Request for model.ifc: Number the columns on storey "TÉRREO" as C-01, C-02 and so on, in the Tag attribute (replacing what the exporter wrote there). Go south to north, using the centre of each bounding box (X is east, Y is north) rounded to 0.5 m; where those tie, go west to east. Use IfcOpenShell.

First a look at what the model holds.

```python
import ifcopenshell
import ifcopenshell.util.element
import ifcopenshell.util.placement

model = ifcopenshell.open("model.ifc")
print(model.schema)
storey = next(s for s in model.by_type("IfcBuildingStorey") if s.Name == "TÉRREO")
columns = [e for e in ifcopenshell.util.element.get_decomposition(storey) if e.is_a("IfcColumn")]
for e in sorted(columns, key=lambda e: e.id()):
    origin = ifcopenshell.util.placement.get_local_placement(e.ObjectPlacement)[:3, 3]
    print(e.id(), e.Tag, e.Name, origin.round(2) + 0.0, sep=" | ")
```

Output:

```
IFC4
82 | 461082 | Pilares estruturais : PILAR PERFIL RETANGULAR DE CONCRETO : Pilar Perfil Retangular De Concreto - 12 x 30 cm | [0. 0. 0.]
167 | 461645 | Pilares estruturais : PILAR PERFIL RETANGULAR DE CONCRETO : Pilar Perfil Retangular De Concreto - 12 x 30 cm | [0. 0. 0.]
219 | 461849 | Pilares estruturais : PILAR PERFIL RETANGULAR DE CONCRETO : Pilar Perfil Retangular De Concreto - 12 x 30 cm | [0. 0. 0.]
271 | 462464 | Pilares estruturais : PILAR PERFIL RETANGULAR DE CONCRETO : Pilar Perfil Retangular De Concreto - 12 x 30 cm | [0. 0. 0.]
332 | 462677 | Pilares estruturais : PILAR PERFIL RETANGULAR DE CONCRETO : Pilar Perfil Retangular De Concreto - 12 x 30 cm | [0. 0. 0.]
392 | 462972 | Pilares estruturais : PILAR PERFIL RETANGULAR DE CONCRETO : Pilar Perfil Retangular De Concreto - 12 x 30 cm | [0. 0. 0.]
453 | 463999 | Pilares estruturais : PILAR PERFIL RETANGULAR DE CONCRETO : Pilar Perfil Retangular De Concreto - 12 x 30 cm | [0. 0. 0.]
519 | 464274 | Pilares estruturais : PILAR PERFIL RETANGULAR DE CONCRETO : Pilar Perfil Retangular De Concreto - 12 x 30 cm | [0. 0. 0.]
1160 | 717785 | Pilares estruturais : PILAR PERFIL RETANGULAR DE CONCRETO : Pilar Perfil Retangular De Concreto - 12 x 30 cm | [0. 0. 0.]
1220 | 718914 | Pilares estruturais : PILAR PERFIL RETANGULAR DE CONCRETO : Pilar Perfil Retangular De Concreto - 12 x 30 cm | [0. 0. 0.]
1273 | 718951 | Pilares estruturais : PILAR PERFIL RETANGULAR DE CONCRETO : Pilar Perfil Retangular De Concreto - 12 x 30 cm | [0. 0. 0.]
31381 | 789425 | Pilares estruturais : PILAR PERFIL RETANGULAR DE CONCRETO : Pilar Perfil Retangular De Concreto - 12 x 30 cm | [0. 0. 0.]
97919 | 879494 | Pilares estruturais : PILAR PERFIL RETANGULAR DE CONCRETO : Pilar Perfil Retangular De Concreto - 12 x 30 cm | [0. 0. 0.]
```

```python
import ifcopenshell
import ifcopenshell.geom
import ifcopenshell.util.element
import ifcopenshell.util.shape

model = ifcopenshell.open("model.ifc")
settings = ifcopenshell.geom.settings()
settings.set("use-world-coords", True)


def centre(element):
    shape = ifcopenshell.geom.create_shape(settings, element)
    return ifcopenshell.util.shape.get_bbox_centroid(shape.geometry)


storey = next(s for s in model.by_type("IfcBuildingStorey") if s.Name == "TÉRREO")
columns = [e for e in ifcopenshell.util.element.get_decomposition(storey) if e.is_a("IfcColumn")]

# Insertion points can sit at a corner or the storey origin, so sort by the geometry (in metres).
centres = {e: centre(e) for e in columns}
columns.sort(key=lambda e: (round(centres[e][1] / 0.5), centres[e][0]))

for i, e in enumerate(columns, start=1):
    number = f"C-{i:02d}"
    e.Tag = number
    print(e.id(), number)

model.write("model-out.ifc")
```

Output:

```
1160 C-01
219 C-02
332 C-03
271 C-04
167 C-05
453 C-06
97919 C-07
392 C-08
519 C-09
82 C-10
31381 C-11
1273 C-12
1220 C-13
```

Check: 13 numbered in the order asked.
